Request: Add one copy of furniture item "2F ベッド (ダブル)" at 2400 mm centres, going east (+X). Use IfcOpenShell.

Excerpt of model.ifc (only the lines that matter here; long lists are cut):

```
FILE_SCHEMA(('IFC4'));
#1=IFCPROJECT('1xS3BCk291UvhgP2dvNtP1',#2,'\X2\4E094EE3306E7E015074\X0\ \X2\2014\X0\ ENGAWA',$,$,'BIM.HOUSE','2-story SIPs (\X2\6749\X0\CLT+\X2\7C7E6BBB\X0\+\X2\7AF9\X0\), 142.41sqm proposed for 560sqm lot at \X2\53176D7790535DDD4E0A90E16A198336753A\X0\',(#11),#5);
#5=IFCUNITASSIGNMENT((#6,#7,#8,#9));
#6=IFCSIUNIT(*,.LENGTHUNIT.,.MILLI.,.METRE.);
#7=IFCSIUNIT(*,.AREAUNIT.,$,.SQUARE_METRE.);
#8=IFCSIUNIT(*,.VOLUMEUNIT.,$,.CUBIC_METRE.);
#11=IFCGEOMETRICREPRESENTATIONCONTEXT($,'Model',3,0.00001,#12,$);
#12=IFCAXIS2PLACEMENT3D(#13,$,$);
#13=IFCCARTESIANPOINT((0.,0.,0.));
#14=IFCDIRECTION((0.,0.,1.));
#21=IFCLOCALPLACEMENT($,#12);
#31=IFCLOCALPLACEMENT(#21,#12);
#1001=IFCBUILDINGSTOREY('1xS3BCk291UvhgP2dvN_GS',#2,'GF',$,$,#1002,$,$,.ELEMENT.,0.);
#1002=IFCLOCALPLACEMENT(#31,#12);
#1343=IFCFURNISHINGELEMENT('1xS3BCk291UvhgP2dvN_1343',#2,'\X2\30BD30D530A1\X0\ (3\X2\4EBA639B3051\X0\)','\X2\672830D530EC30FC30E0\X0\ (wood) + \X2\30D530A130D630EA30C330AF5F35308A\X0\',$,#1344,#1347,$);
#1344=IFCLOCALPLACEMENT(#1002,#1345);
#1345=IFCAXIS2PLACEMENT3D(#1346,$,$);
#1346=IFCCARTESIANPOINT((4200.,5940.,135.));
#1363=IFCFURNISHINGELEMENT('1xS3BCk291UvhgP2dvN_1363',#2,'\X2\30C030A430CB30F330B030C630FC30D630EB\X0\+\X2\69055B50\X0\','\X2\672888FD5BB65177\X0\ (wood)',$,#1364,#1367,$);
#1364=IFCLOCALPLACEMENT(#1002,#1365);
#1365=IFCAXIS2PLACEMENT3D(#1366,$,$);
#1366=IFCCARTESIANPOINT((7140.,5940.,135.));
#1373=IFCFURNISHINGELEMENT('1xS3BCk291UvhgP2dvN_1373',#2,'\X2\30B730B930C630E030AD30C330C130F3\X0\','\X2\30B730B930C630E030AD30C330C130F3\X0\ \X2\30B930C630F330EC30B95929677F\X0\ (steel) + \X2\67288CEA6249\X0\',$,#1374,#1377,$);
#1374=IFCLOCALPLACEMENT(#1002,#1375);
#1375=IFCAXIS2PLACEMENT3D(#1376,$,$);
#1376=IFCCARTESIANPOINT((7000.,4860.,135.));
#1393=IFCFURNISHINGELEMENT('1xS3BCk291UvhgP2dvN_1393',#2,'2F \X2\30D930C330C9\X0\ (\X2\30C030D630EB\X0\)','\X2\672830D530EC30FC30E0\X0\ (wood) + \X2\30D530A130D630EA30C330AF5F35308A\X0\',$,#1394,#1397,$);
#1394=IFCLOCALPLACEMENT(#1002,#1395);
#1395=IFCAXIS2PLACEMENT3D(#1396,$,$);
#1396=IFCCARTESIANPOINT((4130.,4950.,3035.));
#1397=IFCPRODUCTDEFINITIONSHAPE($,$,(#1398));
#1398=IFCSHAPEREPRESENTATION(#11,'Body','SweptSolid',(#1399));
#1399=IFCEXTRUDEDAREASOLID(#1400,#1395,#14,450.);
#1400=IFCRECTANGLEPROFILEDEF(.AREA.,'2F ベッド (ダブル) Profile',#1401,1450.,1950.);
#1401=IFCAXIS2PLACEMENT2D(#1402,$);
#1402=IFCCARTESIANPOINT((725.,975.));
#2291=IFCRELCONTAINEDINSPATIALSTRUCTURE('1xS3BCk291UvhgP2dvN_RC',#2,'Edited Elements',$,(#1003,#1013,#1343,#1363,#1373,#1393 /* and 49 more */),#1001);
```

```python
import numpy as np
import ifcopenshell
import ifcopenshell.api.geometry
import ifcopenshell.api.root
import ifcopenshell.util.element
import ifcopenshell.util.placement
import ifcopenshell.util.unit

model = ifcopenshell.open("model.ifc")
unit_scale = ifcopenshell.util.unit.calculate_unit_scale(model)


def reuse_history(source, copy):
    """copy_class also copies each property set's owner history, people and application; keep the originals."""
    for rel in copy.IsDefinedBy:
        if rel.is_a("IfcRelDefinesByProperties") and (history := rel.RelatingPropertyDefinition.OwnerHistory):
            rel.RelatingPropertyDefinition.OwnerHistory = source.OwnerHistory
            ifcopenshell.util.element.remove_deep2(model, history)


source = model.by_guid("1xS3BCk291UvhgP2dvN_1393")
base = ifcopenshell.util.placement.get_local_placement(source.ObjectPlacement)
step = np.array([1.0, 0.0, 0.0]) * 2.4 / unit_scale

for i in range(1, 2):
    copy = ifcopenshell.api.root.copy_class(model, product=source)
    copy.Representation = ifcopenshell.util.element.copy_deep(
        model, source.Representation, exclude=["IfcGeometricRepresentationContext", "IfcRepresentationMap"]
    )
    reuse_history(source, copy)
    matrix = base.copy()
    matrix[:3, 3] += i * step
    print("added at", matrix[:3, 3].round(3) + 0.0)
    ifcopenshell.api.geometry.edit_object_placement(model, product=copy, matrix=matrix, is_si=False)

model.write("model_rev.ifc")
```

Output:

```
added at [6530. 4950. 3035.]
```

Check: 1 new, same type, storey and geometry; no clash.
